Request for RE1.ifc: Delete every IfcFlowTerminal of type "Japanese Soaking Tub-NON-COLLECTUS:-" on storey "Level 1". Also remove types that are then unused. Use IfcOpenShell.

First a look at what the model holds.

```python
import ifcopenshell
import ifcopenshell.util.element

model = ifcopenshell.open("RE1.ifc")
print(model.schema)
storey = next(s for s in model.by_type("IfcBuildingStorey") if s.Name == "Level 1")
terminals = [e for e in ifcopenshell.util.element.get_decomposition(storey) if e.is_a("IfcFlowTerminal")]
seen = {}
for e in terminals:
    element_type = ifcopenshell.util.element.get_type(e)
    name = element_type.Name if element_type not in (None, e) else None
    seen[name] = seen.get(name, 0) + 1
for name, count in sorted(seen.items(), key=str):
    print(count, "x", name)
```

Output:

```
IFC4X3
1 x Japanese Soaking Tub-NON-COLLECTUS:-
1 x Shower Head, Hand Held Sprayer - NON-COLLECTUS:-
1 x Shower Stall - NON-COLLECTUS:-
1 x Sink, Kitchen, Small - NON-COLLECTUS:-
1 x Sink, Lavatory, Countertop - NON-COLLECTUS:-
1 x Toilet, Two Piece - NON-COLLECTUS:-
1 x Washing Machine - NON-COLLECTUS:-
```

```python
import ifcopenshell
import ifcopenshell.api.root
import ifcopenshell.util.element

model = ifcopenshell.open("RE1.ifc")

storey = next(s for s in model.by_type("IfcBuildingStorey") if s.Name == "Level 1")
terminals = [e for e in ifcopenshell.util.element.get_decomposition(storey) if e.is_a("IfcFlowTerminal")]
targets = [e for e in terminals if (t := ifcopenshell.util.element.get_type(e)) not in (None, e) and t.Name == "Japanese Soaking Tub-NON-COLLECTUS:-"]
types = {ifcopenshell.util.element.get_type(e) for e in targets} - {None, *targets}

for e in targets:
    ifcopenshell.api.root.remove_product(model, product=e)
print(len(targets), "removed")

unused = [t for t in types if not ifcopenshell.util.element.get_types(t)]
for t in unused:
    ifcopenshell.api.root.remove_product(model, product=t)
print(len(unused), "unused types removed")

model.write("RE1_v2.ifc")
```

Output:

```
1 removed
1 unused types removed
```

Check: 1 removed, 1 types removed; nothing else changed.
